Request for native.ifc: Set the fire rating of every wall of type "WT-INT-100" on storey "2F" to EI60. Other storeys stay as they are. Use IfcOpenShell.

First a look at what the model holds.

```python
import ifcopenshell
import ifcopenshell.util.element

model = ifcopenshell.open("native.ifc")
print(model.schema)
storey = next(s for s in model.by_type("IfcBuildingStorey") if s.Name == "2F")
walls = [e for e in ifcopenshell.util.element.get_decomposition(storey) if e.is_a("IfcWall")]
seen = {}
for e in walls:
    element_type = ifcopenshell.util.element.get_type(e)
    key = (element_type.Name if element_type != e and element_type else None, ifcopenshell.util.element.get_pset(e, "Pset_WallCommon", "FireRating"))
    seen[key] = seen.get(key, 0) + 1
for (name, value), count in sorted(seen.items(), key=str):
    print(count, "x", name, "|", value)
```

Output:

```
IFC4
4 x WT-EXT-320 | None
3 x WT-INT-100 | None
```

```python
import ifcopenshell
import ifcopenshell.api.pset
import ifcopenshell.util.element

model = ifcopenshell.open("native.ifc")

storey = next(s for s in model.by_type("IfcBuildingStorey") if s.Name == "2F")
walls = [e for e in ifcopenshell.util.element.get_decomposition(storey) if e.is_a("IfcWall")]

count = 0
for e in walls:
    element_type = ifcopenshell.util.element.get_type(e)
    if element_type in (None, e) or element_type.Name != "WT-INT-100":
        continue
    # add_pset returns the element's existing set when there is one.
    pset = ifcopenshell.api.pset.add_pset(model, product=e, name="Pset_WallCommon")
    ifcopenshell.api.pset.edit_pset(model, pset=pset, properties={"FireRating": "EI60"})
    count += 1

print(count, "walls updated")

model.write("native_rev.ifc")
```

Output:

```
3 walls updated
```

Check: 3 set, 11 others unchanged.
